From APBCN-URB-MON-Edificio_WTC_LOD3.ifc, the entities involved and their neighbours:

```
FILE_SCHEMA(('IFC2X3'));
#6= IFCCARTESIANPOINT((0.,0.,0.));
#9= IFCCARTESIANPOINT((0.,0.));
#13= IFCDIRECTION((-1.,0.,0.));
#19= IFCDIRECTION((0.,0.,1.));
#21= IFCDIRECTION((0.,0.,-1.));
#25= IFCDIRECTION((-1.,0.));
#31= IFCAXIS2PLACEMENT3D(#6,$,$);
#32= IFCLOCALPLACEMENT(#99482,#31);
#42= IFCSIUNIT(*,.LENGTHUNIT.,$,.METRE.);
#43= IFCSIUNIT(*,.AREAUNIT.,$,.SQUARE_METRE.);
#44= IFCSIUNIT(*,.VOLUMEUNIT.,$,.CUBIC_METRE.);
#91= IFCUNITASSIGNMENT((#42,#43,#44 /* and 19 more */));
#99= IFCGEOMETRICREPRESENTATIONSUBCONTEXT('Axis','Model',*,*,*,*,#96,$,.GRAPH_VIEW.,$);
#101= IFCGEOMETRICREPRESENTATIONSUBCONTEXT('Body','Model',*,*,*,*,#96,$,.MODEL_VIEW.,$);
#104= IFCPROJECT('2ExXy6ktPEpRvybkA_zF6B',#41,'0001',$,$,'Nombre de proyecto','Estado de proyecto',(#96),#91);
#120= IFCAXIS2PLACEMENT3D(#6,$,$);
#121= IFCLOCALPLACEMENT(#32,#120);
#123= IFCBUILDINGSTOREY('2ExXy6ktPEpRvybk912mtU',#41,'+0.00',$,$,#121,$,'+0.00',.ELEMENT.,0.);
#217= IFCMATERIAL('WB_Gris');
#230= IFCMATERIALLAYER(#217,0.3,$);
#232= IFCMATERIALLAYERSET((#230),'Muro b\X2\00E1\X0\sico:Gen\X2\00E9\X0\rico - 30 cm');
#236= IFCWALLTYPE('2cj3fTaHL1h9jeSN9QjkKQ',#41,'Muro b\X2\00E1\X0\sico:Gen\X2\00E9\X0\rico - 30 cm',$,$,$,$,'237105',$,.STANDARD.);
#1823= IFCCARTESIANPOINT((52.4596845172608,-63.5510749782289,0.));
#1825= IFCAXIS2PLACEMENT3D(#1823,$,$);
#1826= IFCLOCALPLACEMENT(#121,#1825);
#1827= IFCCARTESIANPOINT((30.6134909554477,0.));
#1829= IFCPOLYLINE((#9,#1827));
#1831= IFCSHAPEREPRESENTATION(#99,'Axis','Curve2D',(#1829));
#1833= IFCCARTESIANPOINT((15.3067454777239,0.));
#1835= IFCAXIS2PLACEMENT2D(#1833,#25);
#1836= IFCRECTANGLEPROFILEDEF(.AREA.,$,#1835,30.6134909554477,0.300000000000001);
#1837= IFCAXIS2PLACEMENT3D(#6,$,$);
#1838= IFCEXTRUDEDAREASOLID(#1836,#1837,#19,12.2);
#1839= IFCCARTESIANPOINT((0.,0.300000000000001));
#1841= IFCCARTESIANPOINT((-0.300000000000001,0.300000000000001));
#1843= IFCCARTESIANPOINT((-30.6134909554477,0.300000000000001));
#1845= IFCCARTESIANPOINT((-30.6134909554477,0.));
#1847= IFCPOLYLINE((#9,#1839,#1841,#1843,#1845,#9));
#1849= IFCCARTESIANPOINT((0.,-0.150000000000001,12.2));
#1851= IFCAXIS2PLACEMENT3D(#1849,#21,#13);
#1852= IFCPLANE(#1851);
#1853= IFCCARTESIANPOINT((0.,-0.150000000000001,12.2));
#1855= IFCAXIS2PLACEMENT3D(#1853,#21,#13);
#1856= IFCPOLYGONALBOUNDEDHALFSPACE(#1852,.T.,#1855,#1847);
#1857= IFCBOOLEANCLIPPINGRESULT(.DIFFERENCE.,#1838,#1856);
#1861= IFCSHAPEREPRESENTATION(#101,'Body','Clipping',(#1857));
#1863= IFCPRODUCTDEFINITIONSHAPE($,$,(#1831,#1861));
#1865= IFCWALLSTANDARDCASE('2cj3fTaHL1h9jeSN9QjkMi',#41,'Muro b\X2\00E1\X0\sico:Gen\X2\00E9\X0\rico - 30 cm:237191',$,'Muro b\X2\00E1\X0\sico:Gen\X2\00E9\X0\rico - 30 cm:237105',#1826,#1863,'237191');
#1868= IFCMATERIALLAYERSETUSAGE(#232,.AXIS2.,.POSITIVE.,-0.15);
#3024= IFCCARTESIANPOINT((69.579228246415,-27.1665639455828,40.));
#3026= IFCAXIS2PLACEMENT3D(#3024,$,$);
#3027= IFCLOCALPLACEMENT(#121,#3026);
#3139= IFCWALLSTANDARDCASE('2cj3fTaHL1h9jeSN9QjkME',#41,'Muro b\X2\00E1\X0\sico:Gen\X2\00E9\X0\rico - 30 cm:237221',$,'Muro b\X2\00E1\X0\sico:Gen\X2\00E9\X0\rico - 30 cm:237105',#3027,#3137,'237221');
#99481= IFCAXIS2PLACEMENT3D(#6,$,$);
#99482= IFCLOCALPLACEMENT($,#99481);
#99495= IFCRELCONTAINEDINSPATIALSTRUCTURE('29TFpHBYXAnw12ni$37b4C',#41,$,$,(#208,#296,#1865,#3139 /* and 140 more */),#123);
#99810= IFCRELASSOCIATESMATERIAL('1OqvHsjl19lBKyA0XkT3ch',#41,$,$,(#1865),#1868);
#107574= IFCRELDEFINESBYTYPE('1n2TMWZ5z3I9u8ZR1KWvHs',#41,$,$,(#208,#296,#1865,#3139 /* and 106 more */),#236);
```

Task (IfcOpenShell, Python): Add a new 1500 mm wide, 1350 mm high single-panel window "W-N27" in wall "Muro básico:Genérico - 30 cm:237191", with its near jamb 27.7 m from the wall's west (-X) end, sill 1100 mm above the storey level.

```python
import numpy as np
import ifcopenshell
import ifcopenshell.api.feature
import ifcopenshell.api.geometry
import ifcopenshell.api.root
import ifcopenshell.api.spatial
import ifcopenshell.api.type
import ifcopenshell.geom
import ifcopenshell.util.element
import ifcopenshell.util.placement
import ifcopenshell.util.representation
import ifcopenshell.util.shape
import ifcopenshell.util.unit

model = ifcopenshell.open("APBCN-URB-MON-Edificio_WTC_LOD3.ifc")
unit_scale = ifcopenshell.util.unit.calculate_unit_scale(model)
settings = ifcopenshell.geom.settings()


def volume(element):
    """Net volume in cubic metres, openings subtracted."""
    shape = ifcopenshell.geom.create_shape(settings, element)
    return ifcopenshell.util.shape.get_volume(shape.geometry)


wall = model.by_id(1865)
storey = ifcopenshell.util.element.get_container(wall, ifc_class="IfcBuildingStorey")
context = ifcopenshell.util.representation.get_context(model, "Model", "Body", "MODEL_VIEW")
before = volume(wall)

width, height, from_end, sill = 1.5, 1.35, 27.7, 1.1  # metres

# The wall runs along its own X axis, and the end named is its -X end.
wall_shape = ifcopenshell.geom.create_shape(settings, wall)
x, y, z = ifcopenshell.util.shape.get_vertices(wall_shape.geometry).T
start = x.min() + from_end
face, thickness = float(y.min()), float(y.max() - y.min())
wall_matrix = ifcopenshell.util.placement.get_local_placement(wall.ObjectPlacement)
level = ifcopenshell.util.placement.get_local_placement(storey.ObjectPlacement)[2, 3]


def in_wall(x, y):
    """Placement at x, y metres in the wall's axes, at sill height."""
    matrix = wall_matrix.copy()
    matrix[:, 3] = wall_matrix @ np.array([x / unit_scale, y / unit_scale, 0.0, 1.0])
    matrix[2, 3] = level + sill / unit_scale
    return matrix


# Opening: a box that overshoots both wall faces by 50 mm.
opening = ifcopenshell.api.root.create_entity(model, ifc_class="IfcOpeningElement")
box = ifcopenshell.api.geometry.add_wall_representation(
    model, context=context, length=width, height=height, thickness=thickness + 0.1
)
ifcopenshell.api.geometry.assign_representation(model, product=opening, representation=box)
ifcopenshell.api.geometry.edit_object_placement(model, product=opening, matrix=in_wall(start, face - 0.05), is_si=False)
ifcopenshell.api.feature.add_feature(model, feature=opening, element=wall)

window = ifcopenshell.api.root.create_entity(model, ifc_class="IfcWindow", name="W-N27")
window.OverallWidth, window.OverallHeight = width / unit_scale, height / unit_scale
body = ifcopenshell.api.geometry.add_window_representation(
    model,
    context=context,
    overall_width=window.OverallWidth,
    overall_height=window.OverallHeight,
    partition_type="SINGLE_PANEL",
)
ifcopenshell.api.geometry.assign_representation(model, product=window, representation=body)
ifcopenshell.api.spatial.assign_container(model, products=[window], relating_structure=storey)
fills = ifcopenshell.api.feature.add_filling(model, opening=opening, element=window)
fills.OwnerHistory = window.OwnerHistory  # required in IFC2X3

# IFC2X3 keeps the operation on the window style.
style = ifcopenshell.api.root.create_entity(model, ifc_class="IfcWindowStyle", name="W-N27")
style.OperationType, style.ConstructionType = "SINGLE_PANEL", "NOTDEFINED"
style.ParameterTakesPrecedence = style.Sizeable = False
ifcopenshell.api.type.assign_type(model, related_objects=[window], relating_type=style)

# Centre the window in the wall's thickness.
ifcopenshell.api.geometry.edit_object_placement(model, product=window, matrix=in_wall(start, face), is_si=False)
window_shape = ifcopenshell.geom.create_shape(settings, window)
depth = ifcopenshell.util.shape.get_vertices(window_shape.geometry)[:, 1]
offset = face + thickness / 2 - (depth.min() + depth.max()) / 2
ifcopenshell.api.geometry.edit_object_placement(model, product=window, matrix=in_wall(start, offset), is_si=False)

after = volume(wall)

print(f"wall volume {before:.3f} -> {after:.3f} m3")

model.write("APBCN-URB-MON-Edificio_WTC_LOD3_updated.ifc")
```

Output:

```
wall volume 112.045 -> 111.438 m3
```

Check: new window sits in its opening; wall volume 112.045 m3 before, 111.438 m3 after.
